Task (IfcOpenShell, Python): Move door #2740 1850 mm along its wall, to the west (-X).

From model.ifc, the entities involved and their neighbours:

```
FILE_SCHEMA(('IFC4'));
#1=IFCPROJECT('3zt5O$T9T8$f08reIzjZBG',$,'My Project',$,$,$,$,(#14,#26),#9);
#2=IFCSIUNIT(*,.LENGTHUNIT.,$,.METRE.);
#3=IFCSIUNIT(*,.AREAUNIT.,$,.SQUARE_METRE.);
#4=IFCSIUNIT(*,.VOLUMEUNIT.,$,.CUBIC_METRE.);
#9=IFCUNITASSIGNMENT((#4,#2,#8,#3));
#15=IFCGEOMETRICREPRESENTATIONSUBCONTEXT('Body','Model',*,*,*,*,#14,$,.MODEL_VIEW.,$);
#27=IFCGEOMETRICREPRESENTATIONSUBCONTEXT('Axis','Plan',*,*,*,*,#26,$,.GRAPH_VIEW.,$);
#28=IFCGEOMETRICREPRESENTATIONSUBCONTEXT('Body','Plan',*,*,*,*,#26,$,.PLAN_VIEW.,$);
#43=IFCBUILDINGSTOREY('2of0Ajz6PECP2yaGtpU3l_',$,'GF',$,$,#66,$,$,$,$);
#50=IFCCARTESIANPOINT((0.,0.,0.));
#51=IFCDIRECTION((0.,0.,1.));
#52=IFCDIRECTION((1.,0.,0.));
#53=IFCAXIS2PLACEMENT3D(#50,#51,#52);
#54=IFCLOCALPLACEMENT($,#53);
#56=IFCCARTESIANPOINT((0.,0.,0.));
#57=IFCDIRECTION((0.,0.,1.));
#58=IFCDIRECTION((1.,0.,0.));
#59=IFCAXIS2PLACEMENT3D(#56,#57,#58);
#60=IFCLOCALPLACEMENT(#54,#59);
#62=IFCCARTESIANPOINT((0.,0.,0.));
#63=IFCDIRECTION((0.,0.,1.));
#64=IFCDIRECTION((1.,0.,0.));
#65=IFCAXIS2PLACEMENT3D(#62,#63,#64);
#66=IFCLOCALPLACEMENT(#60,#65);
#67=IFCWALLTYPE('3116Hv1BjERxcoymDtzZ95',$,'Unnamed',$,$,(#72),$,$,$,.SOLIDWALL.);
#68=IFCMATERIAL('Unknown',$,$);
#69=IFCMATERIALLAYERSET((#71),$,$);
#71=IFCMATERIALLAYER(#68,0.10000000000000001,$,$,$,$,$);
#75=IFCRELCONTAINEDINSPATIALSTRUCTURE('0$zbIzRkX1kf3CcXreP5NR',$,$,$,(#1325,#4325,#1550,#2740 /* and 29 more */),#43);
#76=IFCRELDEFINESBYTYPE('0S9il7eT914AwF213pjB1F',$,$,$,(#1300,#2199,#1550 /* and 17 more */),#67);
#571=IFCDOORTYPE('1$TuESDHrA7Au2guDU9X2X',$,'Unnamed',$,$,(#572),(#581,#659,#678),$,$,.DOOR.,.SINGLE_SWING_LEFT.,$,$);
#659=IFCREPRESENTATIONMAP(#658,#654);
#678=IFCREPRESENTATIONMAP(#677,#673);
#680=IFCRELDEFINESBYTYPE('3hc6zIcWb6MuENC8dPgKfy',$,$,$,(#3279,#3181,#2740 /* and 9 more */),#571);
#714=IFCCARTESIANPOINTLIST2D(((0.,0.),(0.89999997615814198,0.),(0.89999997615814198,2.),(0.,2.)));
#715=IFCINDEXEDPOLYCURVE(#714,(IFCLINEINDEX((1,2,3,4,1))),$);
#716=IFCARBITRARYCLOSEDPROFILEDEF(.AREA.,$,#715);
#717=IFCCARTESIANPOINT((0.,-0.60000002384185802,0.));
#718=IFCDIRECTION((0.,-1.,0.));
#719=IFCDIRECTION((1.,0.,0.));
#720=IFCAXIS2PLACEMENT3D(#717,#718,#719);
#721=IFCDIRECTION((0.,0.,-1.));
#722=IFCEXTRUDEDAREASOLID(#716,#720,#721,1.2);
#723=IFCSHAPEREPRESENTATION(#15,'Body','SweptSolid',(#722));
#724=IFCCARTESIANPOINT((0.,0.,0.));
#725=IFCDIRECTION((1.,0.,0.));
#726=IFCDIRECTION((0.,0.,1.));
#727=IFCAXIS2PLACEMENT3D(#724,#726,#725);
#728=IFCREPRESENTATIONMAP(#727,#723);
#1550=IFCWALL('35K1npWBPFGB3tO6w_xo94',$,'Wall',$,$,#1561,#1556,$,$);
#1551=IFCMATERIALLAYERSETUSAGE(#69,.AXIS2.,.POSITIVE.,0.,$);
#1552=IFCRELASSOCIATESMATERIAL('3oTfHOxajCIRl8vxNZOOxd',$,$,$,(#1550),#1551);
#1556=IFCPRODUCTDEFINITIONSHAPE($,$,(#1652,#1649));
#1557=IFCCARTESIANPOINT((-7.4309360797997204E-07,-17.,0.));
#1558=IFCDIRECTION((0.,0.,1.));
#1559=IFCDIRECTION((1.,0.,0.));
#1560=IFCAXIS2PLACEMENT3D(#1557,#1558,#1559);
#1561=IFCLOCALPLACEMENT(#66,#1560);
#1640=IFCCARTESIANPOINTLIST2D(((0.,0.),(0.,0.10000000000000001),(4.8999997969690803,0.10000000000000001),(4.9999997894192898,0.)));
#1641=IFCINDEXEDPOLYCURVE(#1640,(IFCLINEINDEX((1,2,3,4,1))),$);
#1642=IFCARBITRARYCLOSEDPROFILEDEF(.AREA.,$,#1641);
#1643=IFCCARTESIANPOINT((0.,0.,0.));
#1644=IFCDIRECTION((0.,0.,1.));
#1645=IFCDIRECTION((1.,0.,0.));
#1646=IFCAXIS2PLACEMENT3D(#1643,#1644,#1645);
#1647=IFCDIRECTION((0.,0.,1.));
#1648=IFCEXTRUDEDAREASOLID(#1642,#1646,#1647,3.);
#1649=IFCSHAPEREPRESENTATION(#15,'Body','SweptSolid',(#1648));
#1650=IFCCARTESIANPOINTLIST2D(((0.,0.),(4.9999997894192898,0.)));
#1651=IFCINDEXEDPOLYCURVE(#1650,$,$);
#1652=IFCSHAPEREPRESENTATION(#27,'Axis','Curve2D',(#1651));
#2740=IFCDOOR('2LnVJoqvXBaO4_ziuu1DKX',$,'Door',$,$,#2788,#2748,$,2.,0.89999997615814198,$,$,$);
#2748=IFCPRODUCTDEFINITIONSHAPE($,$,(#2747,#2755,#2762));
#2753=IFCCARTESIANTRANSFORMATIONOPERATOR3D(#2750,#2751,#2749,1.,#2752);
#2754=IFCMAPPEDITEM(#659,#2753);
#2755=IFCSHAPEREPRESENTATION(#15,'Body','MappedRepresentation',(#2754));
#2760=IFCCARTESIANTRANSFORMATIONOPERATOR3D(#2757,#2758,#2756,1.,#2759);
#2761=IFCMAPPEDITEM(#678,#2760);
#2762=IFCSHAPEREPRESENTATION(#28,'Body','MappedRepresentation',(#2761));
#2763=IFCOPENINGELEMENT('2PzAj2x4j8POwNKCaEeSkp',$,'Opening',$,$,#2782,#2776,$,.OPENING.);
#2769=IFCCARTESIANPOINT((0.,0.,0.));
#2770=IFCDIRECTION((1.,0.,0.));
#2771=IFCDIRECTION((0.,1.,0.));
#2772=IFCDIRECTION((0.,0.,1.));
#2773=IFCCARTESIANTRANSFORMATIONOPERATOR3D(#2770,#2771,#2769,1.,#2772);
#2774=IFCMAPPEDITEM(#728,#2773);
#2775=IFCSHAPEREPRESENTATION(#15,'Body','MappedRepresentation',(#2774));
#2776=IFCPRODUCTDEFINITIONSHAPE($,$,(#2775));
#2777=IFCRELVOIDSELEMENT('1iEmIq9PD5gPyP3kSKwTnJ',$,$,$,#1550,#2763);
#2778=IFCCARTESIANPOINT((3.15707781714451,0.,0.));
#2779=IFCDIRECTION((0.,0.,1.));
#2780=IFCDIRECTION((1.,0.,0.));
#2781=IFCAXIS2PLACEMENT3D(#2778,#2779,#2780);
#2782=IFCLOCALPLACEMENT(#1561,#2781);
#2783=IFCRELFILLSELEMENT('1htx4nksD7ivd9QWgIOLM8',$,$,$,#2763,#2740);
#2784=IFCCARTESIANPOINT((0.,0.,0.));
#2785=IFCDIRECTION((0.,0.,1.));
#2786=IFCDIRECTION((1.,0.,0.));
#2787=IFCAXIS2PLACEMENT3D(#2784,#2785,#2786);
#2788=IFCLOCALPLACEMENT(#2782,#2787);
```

```python
import ifcopenshell
import ifcopenshell.api.geometry
import ifcopenshell.util.placement
import ifcopenshell.util.unit

model = ifcopenshell.open("model.ifc")
unit_scale = ifcopenshell.util.unit.calculate_unit_scale(model)

door = model.by_guid("2LnVJoqvXBaO4_ziuu1DKX")
opening = door.FillsVoids[0].RelatingOpeningElement
wall = opening.VoidsElements[0].RelatingBuildingElement

wall_matrix = ifcopenshell.util.placement.get_local_placement(wall.ObjectPlacement)
shift = wall_matrix[:3, 0] * -1.85 / unit_scale
before = ifcopenshell.util.placement.get_local_placement(door.ObjectPlacement)[:3, 3].copy()

# The door is placed relative to its opening, so it follows when the opening moves.
matrix = ifcopenshell.util.placement.get_local_placement(opening.ObjectPlacement)
matrix[:3, 3] += shift
ifcopenshell.api.geometry.edit_object_placement(
    model, product=opening, matrix=matrix, is_si=False, should_transform_children=True
)

after = ifcopenshell.util.placement.get_local_placement(door.ObjectPlacement)[:3, 3]
print("door moved by", (after - before).round(3) + 0.0)

model.write("model-out.ifc")
```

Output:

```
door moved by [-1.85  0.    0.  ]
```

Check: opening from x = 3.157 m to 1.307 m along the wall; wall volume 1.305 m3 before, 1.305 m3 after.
